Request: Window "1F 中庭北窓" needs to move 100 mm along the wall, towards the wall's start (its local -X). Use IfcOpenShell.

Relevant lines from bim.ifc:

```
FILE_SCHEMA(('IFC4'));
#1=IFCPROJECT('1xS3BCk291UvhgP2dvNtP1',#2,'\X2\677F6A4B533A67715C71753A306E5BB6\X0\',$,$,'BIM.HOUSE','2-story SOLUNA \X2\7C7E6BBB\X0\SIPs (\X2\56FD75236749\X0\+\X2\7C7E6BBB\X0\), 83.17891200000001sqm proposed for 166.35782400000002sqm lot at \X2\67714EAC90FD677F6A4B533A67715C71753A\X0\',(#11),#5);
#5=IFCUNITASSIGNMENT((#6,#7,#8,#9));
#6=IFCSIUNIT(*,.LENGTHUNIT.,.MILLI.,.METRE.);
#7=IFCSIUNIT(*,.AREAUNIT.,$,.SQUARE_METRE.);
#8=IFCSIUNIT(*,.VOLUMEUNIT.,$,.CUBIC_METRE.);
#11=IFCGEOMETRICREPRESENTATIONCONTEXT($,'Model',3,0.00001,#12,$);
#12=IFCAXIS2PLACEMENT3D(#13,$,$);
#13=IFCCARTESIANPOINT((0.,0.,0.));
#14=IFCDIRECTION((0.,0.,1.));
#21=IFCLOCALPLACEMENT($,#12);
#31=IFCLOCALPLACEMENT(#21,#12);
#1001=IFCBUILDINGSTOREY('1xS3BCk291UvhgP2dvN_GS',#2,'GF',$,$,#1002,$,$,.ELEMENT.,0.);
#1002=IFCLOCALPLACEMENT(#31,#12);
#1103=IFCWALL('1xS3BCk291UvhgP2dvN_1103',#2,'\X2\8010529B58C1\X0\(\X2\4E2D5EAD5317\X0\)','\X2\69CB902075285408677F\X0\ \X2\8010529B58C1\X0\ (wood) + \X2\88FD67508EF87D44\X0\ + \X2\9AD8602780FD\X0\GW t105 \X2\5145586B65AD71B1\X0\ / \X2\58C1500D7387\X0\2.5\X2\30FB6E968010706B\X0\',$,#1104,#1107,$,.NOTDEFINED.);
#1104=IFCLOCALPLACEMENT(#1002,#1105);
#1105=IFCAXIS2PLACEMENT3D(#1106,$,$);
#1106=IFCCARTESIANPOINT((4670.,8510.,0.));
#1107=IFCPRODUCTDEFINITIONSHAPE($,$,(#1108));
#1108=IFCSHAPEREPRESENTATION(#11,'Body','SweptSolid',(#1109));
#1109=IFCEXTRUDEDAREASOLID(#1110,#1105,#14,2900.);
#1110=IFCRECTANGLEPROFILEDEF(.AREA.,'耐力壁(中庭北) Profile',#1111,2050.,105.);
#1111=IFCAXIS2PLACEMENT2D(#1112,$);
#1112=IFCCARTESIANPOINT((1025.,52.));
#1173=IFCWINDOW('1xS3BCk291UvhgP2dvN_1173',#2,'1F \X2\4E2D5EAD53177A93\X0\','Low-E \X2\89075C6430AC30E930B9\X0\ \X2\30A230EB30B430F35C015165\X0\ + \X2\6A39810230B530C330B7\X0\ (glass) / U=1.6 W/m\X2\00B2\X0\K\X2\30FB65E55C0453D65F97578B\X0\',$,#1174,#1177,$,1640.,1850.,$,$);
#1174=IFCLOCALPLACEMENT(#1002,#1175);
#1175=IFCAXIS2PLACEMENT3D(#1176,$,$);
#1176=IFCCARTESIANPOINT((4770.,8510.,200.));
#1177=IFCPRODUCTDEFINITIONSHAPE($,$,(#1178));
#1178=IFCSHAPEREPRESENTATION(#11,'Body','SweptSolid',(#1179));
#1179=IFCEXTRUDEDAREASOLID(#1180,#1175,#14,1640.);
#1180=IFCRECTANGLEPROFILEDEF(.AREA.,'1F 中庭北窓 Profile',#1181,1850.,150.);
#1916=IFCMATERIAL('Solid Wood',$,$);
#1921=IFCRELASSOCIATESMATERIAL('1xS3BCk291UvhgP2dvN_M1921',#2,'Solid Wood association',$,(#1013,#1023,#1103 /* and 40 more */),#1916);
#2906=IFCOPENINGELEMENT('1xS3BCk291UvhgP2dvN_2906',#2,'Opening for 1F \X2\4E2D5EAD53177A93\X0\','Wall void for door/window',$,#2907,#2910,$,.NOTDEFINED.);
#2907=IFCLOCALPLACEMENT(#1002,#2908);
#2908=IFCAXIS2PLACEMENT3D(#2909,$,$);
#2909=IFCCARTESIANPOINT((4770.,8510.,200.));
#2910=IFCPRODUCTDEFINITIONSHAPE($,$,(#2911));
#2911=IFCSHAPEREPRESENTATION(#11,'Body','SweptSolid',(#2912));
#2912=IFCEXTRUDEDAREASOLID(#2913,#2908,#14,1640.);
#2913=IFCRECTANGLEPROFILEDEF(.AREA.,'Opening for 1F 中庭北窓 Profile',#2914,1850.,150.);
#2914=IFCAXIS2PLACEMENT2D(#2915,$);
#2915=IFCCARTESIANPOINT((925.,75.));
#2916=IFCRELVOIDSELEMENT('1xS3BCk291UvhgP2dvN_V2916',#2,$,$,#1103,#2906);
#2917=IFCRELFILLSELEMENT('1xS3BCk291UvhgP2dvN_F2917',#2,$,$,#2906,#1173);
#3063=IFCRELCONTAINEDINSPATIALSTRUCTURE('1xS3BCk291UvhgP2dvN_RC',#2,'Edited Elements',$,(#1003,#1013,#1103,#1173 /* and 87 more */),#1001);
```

```python
import ifcopenshell
import ifcopenshell.api.geometry
import ifcopenshell.util.placement
import ifcopenshell.util.unit

model = ifcopenshell.open("bim.ifc")
unit_scale = ifcopenshell.util.unit.calculate_unit_scale(model)

window = model.by_guid("1xS3BCk291UvhgP2dvN_1173")
opening = window.FillsVoids[0].RelatingOpeningElement
wall = opening.VoidsElements[0].RelatingBuildingElement

wall_matrix = ifcopenshell.util.placement.get_local_placement(wall.ObjectPlacement)
shift = wall_matrix[:3, 0] * -0.1 / unit_scale
before = ifcopenshell.util.placement.get_local_placement(window.ObjectPlacement)[:3, 3].copy()

# The window is not placed relative to its opening, so move both.
for product in (opening, window):
    matrix = ifcopenshell.util.placement.get_local_placement(product.ObjectPlacement)
    matrix[:3, 3] += shift
    ifcopenshell.api.geometry.edit_object_placement(model, product=product, matrix=matrix, is_si=False)

after = ifcopenshell.util.placement.get_local_placement(window.ObjectPlacement)[:3, 3]
print("window moved by", (after - before).round(3) + 0.0)

model.write("bim_v2.ifc")
```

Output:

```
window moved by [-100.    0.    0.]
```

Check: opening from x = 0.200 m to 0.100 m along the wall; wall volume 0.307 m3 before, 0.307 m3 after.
